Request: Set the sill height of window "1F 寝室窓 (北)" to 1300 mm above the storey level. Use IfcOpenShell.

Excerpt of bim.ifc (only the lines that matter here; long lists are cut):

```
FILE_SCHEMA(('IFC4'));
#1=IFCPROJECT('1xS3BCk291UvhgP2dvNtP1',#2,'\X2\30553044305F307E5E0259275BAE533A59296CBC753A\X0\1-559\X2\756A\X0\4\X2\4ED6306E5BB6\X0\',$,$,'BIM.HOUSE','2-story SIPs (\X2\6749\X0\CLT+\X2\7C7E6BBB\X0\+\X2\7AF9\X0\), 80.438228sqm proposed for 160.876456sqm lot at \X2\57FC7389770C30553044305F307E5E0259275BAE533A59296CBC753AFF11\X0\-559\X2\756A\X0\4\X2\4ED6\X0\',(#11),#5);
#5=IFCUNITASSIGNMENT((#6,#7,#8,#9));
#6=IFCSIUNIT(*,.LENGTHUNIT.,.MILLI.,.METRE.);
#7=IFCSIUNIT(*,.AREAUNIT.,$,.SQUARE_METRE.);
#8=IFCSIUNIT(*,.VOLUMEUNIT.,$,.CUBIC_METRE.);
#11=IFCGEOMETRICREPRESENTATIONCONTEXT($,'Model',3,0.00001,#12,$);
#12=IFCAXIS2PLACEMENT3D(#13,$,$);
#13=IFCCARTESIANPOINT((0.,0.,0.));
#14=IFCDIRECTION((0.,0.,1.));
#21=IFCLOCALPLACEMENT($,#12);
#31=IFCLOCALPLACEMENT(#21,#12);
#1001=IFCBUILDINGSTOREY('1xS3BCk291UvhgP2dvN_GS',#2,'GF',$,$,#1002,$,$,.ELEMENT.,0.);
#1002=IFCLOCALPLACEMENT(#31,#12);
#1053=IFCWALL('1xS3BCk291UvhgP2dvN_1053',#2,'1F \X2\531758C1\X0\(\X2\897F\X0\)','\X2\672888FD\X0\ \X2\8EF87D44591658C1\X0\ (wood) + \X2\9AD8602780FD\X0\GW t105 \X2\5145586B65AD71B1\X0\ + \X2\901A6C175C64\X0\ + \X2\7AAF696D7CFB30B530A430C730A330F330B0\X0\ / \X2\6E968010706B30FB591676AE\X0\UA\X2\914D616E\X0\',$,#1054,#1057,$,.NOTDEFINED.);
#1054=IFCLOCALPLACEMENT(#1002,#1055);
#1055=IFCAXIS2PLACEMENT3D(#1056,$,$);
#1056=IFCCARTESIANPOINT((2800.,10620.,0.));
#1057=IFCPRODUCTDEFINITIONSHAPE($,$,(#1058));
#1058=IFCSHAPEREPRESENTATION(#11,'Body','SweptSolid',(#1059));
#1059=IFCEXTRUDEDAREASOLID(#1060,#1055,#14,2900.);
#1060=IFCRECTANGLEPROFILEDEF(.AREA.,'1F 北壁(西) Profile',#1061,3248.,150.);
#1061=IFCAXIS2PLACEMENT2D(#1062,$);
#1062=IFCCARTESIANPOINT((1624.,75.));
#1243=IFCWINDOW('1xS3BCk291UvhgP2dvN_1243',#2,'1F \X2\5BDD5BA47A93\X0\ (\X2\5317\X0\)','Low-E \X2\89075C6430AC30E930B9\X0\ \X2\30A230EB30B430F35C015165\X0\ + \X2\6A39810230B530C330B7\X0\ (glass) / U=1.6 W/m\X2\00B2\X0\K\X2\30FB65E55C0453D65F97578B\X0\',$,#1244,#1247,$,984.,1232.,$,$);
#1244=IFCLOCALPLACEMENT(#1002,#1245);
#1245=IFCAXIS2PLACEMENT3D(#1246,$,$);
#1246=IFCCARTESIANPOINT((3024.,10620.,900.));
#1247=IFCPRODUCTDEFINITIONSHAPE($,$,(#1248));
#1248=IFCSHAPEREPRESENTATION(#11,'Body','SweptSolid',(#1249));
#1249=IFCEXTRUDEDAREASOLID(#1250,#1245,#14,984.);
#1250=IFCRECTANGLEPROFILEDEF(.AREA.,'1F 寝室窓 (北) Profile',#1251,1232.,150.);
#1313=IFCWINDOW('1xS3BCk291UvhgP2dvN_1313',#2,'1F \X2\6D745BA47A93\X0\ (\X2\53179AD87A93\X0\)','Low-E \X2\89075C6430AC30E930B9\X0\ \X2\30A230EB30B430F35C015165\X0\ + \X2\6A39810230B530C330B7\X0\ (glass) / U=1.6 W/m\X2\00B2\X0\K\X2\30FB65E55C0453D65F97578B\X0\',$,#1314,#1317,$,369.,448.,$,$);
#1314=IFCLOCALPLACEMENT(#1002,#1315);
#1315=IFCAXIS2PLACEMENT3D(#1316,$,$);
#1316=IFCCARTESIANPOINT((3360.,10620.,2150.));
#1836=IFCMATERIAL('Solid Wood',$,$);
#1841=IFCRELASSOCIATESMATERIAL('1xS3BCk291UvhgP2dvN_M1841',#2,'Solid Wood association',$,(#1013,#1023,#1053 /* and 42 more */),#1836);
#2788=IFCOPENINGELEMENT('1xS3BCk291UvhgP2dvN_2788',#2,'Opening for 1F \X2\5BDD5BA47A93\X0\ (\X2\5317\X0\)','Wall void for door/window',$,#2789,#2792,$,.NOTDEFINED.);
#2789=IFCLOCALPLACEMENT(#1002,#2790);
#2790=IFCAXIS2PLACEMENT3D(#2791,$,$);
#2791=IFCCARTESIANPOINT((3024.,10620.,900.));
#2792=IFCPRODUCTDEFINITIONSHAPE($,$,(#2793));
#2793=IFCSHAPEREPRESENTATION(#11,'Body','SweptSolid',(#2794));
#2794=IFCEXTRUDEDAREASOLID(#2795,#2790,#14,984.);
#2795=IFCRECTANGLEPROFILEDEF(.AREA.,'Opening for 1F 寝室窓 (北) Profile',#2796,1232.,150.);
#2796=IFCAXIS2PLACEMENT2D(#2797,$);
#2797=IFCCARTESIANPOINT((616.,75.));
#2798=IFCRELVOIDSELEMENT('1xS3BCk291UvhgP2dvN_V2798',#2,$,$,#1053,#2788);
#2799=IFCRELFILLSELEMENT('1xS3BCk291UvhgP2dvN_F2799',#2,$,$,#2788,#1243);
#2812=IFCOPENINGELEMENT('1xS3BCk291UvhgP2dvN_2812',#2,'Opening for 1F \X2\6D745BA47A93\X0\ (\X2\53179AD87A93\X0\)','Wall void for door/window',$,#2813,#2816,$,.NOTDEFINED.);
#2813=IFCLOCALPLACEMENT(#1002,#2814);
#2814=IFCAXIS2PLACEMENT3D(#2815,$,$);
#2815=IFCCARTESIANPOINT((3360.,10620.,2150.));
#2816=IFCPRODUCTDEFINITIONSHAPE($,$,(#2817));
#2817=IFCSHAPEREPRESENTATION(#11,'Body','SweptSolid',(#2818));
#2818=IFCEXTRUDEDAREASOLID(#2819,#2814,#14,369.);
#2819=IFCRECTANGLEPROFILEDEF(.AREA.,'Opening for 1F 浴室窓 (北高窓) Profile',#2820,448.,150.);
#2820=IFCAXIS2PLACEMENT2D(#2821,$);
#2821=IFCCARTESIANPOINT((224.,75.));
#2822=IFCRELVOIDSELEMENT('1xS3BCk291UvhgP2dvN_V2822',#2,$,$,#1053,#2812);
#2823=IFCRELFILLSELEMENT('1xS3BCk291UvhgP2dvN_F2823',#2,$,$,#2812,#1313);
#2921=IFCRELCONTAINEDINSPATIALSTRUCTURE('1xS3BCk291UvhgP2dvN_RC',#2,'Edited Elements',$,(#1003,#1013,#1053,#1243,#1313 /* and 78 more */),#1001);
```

```python
import numpy as np
import ifcopenshell
import ifcopenshell.api.geometry
import ifcopenshell.geom
import ifcopenshell.util.element
import ifcopenshell.util.placement
import ifcopenshell.util.shape
import ifcopenshell.util.unit

model = ifcopenshell.open("bim.ifc")
unit_scale = ifcopenshell.util.unit.calculate_unit_scale(model)

window = model.by_id(1243)
opening = window.FillsVoids[0].RelatingOpeningElement
storey = ifcopenshell.util.element.get_container(window, ifc_class="IfcBuildingStorey")
level = ifcopenshell.util.placement.get_local_placement(storey.ObjectPlacement)[2, 3]

# The opening's origin need not be at the sill, so measure its lowest point.
shape = ifcopenshell.geom.create_shape(ifcopenshell.geom.settings(), opening)
bottom = ifcopenshell.util.shape.get_shape_bottom_elevation(shape, shape.geometry) / unit_scale
dz = level + 1300.0 - bottom

shift = np.array([0.0, 0.0, dz])
# The window is not placed relative to its opening, so move both.
for product in (opening, window):
    matrix = ifcopenshell.util.placement.get_local_placement(product.ObjectPlacement)
    matrix[:3, 3] += shift
    ifcopenshell.api.geometry.edit_object_placement(model, product=product, matrix=matrix, is_si=False)

print(f"moved by {dz * unit_scale:+.3f} m")

model.write("bim_v2.ifc")
```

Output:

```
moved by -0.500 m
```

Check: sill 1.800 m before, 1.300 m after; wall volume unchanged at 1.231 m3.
